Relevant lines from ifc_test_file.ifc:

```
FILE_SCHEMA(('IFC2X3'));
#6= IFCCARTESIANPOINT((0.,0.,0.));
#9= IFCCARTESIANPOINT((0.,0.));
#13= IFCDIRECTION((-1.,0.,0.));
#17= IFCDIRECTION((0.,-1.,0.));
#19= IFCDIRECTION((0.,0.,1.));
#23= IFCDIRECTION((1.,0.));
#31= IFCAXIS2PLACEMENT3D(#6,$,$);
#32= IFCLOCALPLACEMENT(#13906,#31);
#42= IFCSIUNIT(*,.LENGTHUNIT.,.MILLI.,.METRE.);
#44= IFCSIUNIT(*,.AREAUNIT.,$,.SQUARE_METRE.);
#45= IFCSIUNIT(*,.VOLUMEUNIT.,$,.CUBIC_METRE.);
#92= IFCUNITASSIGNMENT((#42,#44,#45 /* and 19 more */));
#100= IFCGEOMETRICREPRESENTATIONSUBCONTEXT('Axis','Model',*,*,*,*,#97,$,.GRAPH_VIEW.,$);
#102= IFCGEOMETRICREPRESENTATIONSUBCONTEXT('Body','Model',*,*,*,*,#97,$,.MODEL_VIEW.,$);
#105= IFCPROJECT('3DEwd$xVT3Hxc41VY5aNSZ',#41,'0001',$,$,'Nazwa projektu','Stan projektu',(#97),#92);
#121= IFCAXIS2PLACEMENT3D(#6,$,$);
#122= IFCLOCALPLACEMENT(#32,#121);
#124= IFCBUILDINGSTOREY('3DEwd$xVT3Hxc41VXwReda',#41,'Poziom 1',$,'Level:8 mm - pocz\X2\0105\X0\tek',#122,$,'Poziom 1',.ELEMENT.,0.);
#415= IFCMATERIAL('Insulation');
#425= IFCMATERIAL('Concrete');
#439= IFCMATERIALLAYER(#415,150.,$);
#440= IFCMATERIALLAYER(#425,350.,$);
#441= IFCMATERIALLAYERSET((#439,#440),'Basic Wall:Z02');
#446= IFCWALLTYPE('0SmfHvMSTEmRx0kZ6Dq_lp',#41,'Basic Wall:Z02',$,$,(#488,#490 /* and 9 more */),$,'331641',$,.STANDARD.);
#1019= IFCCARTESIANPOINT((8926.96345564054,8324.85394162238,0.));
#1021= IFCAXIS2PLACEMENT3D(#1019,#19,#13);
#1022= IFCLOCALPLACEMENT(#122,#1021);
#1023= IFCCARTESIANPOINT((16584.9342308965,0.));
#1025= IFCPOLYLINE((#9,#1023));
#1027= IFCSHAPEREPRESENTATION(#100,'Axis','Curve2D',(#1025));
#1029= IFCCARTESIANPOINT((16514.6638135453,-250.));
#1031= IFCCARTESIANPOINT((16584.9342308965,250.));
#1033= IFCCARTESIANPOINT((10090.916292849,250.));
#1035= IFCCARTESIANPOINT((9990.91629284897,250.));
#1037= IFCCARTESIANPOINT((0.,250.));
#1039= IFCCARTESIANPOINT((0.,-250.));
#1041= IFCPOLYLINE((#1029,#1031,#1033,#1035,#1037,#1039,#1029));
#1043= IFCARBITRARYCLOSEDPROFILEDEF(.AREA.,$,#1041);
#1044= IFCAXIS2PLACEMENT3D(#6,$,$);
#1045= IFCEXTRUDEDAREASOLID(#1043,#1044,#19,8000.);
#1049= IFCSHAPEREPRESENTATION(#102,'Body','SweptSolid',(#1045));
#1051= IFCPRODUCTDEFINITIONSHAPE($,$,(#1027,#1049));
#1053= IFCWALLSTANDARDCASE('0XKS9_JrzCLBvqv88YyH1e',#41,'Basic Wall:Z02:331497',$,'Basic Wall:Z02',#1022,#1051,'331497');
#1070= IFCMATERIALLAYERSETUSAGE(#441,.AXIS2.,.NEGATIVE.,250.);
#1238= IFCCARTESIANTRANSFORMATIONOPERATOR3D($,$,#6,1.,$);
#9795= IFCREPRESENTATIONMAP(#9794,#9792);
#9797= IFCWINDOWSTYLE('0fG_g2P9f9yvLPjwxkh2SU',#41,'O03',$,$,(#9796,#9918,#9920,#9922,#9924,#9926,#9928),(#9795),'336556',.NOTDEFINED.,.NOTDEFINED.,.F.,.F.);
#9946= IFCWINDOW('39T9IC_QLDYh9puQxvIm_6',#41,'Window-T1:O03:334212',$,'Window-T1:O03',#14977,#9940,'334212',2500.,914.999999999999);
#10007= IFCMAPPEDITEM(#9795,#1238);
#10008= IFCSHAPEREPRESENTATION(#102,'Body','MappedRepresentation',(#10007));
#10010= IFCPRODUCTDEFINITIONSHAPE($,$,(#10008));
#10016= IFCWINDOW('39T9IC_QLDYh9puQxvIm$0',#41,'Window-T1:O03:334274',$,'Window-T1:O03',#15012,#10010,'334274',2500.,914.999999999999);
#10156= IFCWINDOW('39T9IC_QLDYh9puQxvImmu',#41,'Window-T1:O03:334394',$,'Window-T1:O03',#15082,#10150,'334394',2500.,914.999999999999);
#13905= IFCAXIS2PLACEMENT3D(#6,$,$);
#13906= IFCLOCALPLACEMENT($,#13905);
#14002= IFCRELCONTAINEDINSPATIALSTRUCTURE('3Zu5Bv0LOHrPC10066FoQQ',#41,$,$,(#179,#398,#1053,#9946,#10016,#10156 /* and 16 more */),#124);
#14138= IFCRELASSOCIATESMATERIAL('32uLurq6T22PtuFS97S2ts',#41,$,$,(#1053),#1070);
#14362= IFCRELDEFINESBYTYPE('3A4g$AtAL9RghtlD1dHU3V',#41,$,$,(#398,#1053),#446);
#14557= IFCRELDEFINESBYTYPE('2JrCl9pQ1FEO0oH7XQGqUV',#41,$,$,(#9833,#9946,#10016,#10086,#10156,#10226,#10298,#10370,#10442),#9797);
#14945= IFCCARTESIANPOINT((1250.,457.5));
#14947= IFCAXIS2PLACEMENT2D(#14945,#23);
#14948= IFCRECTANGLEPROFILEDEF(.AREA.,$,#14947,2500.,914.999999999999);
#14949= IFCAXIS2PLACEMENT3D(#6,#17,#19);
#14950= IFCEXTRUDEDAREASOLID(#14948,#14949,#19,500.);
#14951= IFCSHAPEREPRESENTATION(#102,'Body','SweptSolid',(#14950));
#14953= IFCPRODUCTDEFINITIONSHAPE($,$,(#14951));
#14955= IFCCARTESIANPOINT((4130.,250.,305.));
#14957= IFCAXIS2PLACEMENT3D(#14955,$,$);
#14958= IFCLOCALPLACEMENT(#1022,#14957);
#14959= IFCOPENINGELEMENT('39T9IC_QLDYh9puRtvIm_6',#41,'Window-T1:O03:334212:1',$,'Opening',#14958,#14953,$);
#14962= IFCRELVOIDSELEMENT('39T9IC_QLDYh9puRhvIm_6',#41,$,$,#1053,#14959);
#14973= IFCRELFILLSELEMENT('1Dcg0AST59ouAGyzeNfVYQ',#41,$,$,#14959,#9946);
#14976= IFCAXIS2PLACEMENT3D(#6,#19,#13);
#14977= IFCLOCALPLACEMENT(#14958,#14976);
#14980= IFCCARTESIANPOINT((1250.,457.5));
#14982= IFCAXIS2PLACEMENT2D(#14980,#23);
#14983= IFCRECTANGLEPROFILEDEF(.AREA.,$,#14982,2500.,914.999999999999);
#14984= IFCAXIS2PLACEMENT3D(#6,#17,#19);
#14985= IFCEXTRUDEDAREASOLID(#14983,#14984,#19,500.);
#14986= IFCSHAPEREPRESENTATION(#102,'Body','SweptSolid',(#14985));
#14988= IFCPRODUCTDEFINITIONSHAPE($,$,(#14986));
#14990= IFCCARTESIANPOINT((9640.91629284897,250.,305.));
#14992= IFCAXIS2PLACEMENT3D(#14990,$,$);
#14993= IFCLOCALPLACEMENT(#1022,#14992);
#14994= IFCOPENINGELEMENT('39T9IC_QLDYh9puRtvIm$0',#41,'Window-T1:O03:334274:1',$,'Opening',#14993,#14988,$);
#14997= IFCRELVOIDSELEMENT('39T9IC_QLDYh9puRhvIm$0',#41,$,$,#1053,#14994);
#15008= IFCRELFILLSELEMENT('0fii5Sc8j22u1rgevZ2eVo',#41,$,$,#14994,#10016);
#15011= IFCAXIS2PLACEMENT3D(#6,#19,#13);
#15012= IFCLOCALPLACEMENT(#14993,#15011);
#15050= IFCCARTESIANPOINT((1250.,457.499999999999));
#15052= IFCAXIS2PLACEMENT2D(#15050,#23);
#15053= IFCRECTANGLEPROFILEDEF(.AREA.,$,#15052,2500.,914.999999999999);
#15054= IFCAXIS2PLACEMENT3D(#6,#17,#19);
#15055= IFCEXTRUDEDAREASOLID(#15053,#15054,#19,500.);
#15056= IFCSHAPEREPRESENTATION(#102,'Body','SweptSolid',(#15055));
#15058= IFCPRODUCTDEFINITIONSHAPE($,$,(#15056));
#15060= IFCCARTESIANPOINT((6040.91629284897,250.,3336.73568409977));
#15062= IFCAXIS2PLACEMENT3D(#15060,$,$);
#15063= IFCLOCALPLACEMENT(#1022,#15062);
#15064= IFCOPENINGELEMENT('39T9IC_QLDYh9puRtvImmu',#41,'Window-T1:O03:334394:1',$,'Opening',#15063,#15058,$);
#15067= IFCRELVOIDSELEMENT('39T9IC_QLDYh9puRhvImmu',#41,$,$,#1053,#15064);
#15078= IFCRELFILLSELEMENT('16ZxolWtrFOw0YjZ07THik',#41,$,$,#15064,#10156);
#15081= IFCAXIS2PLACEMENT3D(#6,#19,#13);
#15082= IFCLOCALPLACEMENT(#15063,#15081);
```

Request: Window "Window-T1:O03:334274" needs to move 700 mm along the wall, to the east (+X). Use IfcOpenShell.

```python
import ifcopenshell
import ifcopenshell.api.geometry
import ifcopenshell.util.placement
import ifcopenshell.util.unit

model = ifcopenshell.open("ifc_test_file.ifc")
unit_scale = ifcopenshell.util.unit.calculate_unit_scale(model)

window = model.by_id(10016)
opening = window.FillsVoids[0].RelatingOpeningElement
wall = opening.VoidsElements[0].RelatingBuildingElement

wall_matrix = ifcopenshell.util.placement.get_local_placement(wall.ObjectPlacement)
shift = wall_matrix[:3, 0] * -0.7 / unit_scale
before = ifcopenshell.util.placement.get_local_placement(window.ObjectPlacement)[:3, 3].copy()

# The window is placed relative to its opening, so it follows when the opening moves.
matrix = ifcopenshell.util.placement.get_local_placement(opening.ObjectPlacement)
matrix[:3, 3] += shift
ifcopenshell.api.geometry.edit_object_placement(
    model, product=opening, matrix=matrix, is_si=False, should_transform_children=True
)

after = ifcopenshell.util.placement.get_local_placement(window.ObjectPlacement)[:3, 3]
print("window moved by", (after - before).round(3) + 0.0)

model.write("ifc_test_file-out.ifc")
```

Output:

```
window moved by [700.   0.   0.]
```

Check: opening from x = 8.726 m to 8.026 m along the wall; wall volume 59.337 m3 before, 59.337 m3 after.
